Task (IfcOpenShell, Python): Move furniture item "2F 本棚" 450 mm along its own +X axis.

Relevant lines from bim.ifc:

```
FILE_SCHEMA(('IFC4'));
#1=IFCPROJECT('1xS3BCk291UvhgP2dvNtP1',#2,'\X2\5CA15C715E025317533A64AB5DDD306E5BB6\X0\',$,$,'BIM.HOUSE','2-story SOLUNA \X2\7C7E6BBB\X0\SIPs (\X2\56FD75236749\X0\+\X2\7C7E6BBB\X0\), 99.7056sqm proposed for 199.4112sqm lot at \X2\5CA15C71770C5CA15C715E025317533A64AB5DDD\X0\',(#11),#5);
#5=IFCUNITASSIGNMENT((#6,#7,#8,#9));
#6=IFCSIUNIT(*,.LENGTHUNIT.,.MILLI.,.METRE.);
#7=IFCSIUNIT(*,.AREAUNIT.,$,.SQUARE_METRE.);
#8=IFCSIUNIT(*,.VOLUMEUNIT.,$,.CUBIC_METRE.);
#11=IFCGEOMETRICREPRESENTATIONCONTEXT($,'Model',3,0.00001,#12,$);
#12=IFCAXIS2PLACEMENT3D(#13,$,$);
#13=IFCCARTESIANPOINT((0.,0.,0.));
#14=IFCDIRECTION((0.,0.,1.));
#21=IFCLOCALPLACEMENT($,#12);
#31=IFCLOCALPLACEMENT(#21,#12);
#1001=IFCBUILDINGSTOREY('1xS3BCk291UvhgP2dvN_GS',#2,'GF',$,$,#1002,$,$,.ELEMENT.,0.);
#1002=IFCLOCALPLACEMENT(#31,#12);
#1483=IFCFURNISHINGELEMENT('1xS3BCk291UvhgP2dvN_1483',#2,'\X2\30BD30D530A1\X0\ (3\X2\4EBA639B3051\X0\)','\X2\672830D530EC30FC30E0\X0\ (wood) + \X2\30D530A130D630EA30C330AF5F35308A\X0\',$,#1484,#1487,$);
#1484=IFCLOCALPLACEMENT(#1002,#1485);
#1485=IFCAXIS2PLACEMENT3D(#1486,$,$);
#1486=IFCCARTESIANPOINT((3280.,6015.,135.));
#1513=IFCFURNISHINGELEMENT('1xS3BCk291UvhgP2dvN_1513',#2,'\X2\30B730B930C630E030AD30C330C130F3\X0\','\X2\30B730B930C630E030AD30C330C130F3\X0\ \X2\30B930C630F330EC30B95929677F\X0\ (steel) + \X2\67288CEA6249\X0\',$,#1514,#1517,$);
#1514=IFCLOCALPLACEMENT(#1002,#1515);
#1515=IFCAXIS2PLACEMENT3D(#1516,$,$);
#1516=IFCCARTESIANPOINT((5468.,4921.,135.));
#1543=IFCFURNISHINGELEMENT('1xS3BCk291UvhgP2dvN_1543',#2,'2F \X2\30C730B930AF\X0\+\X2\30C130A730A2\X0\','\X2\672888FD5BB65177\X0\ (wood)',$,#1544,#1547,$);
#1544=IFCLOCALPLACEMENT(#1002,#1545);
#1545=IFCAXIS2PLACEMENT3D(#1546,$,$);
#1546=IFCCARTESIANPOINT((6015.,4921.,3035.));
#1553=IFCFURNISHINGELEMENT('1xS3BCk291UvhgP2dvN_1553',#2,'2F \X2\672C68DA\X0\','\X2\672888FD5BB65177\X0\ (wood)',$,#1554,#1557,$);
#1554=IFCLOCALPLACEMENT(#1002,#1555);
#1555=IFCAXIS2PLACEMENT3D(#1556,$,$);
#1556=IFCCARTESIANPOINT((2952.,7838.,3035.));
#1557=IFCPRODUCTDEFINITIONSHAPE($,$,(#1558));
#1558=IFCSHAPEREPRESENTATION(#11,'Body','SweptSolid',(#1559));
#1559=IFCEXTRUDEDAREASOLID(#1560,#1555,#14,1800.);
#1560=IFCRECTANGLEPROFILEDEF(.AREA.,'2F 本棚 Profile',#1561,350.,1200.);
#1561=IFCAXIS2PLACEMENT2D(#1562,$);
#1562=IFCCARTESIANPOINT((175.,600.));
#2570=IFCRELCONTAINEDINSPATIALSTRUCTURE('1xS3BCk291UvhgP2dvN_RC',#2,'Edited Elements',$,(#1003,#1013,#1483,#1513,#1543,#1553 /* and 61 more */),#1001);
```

```python
import ifcopenshell
import ifcopenshell.api.geometry
import ifcopenshell.util.placement

model = ifcopenshell.open("bim.ifc")

item = model.by_guid("1xS3BCk291UvhgP2dvN_1553")
matrix = ifcopenshell.util.placement.get_local_placement(item.ObjectPlacement)
matrix[:3, 3] += matrix[:3, 0] * 450.0
ifcopenshell.api.geometry.edit_object_placement(model, product=item, matrix=matrix, is_si=False)

print(ifcopenshell.util.placement.get_local_placement(item.ObjectPlacement).round(3) + 0.0)

model.write("bim_rev.ifc")
```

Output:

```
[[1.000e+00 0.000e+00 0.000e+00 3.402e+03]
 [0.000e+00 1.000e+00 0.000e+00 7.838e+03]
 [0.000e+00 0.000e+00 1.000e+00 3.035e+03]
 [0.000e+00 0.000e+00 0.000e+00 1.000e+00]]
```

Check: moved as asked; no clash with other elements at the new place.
